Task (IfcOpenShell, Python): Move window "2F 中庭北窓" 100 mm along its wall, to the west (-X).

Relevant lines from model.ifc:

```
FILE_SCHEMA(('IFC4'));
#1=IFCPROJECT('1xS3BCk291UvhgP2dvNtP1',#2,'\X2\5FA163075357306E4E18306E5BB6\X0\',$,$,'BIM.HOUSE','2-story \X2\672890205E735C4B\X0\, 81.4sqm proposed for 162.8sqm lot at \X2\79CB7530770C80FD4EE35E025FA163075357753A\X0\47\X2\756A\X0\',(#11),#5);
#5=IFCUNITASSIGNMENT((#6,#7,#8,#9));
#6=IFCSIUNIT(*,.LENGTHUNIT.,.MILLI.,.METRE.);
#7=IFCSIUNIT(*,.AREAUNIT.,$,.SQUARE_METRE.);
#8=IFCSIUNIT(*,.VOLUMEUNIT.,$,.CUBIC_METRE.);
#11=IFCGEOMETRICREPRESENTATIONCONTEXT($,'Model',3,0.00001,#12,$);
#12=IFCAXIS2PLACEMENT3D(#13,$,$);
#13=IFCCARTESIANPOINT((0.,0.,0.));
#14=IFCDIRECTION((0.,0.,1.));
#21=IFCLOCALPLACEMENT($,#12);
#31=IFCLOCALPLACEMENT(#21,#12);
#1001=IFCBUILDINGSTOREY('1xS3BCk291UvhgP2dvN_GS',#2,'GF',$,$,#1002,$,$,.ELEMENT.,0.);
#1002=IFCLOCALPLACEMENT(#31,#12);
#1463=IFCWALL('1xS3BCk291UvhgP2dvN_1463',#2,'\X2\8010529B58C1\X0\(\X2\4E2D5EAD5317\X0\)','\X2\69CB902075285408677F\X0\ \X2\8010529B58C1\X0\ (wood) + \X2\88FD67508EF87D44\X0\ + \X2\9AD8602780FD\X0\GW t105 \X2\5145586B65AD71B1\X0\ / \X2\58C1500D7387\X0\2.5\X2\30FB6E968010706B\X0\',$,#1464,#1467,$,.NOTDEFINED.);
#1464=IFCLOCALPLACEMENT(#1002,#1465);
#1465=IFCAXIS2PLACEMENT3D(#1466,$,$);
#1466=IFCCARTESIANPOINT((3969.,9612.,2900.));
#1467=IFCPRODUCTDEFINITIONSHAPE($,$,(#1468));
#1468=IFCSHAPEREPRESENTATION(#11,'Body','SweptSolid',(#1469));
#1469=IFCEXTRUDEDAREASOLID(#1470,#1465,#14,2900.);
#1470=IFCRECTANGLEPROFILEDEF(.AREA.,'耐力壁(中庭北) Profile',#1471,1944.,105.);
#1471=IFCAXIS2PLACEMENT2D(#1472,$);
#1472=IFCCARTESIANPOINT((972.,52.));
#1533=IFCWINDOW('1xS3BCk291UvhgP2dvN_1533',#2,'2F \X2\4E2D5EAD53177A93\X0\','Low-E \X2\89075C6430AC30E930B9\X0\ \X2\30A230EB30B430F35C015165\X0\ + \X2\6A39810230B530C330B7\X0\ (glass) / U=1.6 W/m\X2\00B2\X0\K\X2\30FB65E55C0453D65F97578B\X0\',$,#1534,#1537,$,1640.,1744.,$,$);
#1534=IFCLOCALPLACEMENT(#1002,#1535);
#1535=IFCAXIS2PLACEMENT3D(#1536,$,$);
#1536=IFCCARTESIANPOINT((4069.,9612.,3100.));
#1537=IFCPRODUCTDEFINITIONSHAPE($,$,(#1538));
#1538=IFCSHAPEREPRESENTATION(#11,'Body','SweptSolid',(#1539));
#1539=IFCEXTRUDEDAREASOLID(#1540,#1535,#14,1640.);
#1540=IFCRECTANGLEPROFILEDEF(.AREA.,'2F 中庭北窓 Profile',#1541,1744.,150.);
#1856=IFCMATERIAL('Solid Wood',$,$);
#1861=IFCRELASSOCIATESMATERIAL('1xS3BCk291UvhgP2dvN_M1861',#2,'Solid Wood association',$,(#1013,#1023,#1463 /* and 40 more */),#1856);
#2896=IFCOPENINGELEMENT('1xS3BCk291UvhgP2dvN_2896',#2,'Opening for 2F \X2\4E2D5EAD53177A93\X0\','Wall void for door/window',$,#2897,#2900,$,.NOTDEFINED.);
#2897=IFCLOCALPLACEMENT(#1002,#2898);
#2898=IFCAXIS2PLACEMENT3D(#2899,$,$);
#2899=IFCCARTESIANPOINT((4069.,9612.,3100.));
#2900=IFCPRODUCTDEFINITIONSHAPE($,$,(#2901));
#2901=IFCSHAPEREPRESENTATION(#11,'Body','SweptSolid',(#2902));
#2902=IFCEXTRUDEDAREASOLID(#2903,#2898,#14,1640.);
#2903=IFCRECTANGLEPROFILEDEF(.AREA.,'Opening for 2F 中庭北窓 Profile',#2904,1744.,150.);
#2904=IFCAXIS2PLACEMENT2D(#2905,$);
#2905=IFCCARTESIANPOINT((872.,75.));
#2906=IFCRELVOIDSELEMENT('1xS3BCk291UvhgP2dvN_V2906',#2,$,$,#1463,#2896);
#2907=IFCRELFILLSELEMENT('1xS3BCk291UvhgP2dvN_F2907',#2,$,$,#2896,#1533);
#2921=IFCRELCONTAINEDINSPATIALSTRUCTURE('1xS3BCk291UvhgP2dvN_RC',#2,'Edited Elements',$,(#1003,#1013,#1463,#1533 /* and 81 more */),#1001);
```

```python
import ifcopenshell
import ifcopenshell.api.geometry
import ifcopenshell.util.placement
import ifcopenshell.util.unit

model = ifcopenshell.open("model.ifc")
unit_scale = ifcopenshell.util.unit.calculate_unit_scale(model)

window = model.by_guid("1xS3BCk291UvhgP2dvN_1533")
opening = window.FillsVoids[0].RelatingOpeningElement
wall = opening.VoidsElements[0].RelatingBuildingElement

wall_matrix = ifcopenshell.util.placement.get_local_placement(wall.ObjectPlacement)
shift = wall_matrix[:3, 0] * -0.1 / unit_scale
before = ifcopenshell.util.placement.get_local_placement(window.ObjectPlacement)[:3, 3].copy()

# The window is not placed relative to its opening, so move both.
for product in (opening, window):
    matrix = ifcopenshell.util.placement.get_local_placement(product.ObjectPlacement)
    matrix[:3, 3] += shift
    ifcopenshell.api.geometry.edit_object_placement(model, product=product, matrix=matrix, is_si=False)

after = ifcopenshell.util.placement.get_local_placement(window.ObjectPlacement)[:3, 3]
print("window moved by", (after - before).round(3) + 0.0)

model.write("model-out.ifc")
```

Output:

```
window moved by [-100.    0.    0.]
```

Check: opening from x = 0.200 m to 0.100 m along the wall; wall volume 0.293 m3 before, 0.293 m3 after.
